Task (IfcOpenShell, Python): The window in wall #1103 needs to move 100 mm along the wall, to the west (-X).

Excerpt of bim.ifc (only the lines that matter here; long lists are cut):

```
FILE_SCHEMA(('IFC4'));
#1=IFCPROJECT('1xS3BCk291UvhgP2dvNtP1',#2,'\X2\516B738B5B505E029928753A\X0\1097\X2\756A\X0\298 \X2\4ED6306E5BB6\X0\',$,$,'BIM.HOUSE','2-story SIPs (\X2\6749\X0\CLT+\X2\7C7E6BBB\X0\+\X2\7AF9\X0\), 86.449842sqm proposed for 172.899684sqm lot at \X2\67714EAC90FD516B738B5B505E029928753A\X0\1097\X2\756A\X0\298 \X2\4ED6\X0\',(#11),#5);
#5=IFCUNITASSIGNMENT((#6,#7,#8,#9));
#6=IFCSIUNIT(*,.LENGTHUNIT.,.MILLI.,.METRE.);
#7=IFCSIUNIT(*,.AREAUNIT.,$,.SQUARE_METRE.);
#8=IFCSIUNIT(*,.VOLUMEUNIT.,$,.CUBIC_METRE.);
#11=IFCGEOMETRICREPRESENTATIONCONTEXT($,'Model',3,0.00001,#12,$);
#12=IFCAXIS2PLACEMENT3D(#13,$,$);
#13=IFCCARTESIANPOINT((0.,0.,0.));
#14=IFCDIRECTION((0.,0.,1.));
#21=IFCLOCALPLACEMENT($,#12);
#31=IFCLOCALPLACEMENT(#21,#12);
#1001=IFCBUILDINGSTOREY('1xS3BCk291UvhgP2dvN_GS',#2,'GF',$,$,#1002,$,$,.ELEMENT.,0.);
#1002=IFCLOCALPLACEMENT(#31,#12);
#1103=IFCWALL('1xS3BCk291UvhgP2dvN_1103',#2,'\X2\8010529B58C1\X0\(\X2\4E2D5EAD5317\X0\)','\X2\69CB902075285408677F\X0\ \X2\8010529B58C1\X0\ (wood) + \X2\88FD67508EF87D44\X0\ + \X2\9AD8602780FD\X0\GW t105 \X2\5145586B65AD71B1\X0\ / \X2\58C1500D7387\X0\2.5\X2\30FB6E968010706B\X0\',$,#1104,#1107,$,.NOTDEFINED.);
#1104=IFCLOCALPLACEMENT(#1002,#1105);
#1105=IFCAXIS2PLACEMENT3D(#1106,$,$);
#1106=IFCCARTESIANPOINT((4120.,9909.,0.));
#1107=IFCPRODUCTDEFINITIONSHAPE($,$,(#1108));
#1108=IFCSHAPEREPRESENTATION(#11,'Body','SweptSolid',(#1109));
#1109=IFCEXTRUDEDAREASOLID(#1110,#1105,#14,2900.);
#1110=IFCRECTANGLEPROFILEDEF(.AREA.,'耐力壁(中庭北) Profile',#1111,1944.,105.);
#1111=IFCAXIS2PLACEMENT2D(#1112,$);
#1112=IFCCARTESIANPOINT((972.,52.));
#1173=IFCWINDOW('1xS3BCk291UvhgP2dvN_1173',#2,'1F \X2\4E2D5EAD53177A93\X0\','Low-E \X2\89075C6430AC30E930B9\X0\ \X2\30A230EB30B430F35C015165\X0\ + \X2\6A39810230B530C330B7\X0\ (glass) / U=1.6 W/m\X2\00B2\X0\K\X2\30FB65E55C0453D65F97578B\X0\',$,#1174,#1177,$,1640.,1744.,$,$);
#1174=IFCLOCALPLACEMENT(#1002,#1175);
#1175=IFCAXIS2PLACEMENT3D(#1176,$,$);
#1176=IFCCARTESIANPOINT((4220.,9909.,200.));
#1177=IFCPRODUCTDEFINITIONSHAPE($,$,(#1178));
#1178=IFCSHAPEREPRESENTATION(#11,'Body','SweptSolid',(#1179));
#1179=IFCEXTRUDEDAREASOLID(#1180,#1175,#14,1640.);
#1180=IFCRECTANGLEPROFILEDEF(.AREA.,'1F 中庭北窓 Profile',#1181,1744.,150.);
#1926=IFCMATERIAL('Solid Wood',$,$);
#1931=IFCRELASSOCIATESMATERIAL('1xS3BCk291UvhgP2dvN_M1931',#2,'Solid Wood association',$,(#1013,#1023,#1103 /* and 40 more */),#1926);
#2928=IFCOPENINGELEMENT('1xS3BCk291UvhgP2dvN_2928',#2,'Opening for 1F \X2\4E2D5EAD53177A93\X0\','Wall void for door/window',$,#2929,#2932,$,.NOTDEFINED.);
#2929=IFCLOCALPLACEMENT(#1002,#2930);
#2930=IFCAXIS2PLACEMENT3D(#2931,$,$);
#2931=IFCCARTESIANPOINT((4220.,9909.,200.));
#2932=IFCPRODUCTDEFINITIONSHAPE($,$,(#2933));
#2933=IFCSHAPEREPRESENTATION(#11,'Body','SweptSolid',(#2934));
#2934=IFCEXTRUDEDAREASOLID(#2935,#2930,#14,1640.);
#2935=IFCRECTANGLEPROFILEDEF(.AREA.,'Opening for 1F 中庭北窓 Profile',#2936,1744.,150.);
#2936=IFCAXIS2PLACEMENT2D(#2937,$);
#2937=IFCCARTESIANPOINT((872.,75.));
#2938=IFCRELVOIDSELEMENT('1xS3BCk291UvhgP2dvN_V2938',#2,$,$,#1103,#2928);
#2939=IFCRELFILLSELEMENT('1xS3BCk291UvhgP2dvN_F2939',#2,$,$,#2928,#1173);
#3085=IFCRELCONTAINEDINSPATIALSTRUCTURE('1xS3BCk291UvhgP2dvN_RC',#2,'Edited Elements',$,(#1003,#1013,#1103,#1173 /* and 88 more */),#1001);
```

```python
import ifcopenshell
import ifcopenshell.api.geometry
import ifcopenshell.util.placement

model = ifcopenshell.open("bim.ifc")

window = model.by_id(1173)
opening = window.FillsVoids[0].RelatingOpeningElement
wall = opening.VoidsElements[0].RelatingBuildingElement

wall_matrix = ifcopenshell.util.placement.get_local_placement(wall.ObjectPlacement)
shift = wall_matrix[:3, 0] * -100.0
before = ifcopenshell.util.placement.get_local_placement(window.ObjectPlacement)[:3, 3].copy()

# The window is not placed relative to its opening, so move both.
for product in (opening, window):
    matrix = ifcopenshell.util.placement.get_local_placement(product.ObjectPlacement)
    matrix[:3, 3] += shift
    ifcopenshell.api.geometry.edit_object_placement(model, product=product, matrix=matrix, is_si=False)

after = ifcopenshell.util.placement.get_local_placement(window.ObjectPlacement)[:3, 3]
print("window moved by", (after - before).round(3) + 0.0)

model.write("bim_v2.ifc")
```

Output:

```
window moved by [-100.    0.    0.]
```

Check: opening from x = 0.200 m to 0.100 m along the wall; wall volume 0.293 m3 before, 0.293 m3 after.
